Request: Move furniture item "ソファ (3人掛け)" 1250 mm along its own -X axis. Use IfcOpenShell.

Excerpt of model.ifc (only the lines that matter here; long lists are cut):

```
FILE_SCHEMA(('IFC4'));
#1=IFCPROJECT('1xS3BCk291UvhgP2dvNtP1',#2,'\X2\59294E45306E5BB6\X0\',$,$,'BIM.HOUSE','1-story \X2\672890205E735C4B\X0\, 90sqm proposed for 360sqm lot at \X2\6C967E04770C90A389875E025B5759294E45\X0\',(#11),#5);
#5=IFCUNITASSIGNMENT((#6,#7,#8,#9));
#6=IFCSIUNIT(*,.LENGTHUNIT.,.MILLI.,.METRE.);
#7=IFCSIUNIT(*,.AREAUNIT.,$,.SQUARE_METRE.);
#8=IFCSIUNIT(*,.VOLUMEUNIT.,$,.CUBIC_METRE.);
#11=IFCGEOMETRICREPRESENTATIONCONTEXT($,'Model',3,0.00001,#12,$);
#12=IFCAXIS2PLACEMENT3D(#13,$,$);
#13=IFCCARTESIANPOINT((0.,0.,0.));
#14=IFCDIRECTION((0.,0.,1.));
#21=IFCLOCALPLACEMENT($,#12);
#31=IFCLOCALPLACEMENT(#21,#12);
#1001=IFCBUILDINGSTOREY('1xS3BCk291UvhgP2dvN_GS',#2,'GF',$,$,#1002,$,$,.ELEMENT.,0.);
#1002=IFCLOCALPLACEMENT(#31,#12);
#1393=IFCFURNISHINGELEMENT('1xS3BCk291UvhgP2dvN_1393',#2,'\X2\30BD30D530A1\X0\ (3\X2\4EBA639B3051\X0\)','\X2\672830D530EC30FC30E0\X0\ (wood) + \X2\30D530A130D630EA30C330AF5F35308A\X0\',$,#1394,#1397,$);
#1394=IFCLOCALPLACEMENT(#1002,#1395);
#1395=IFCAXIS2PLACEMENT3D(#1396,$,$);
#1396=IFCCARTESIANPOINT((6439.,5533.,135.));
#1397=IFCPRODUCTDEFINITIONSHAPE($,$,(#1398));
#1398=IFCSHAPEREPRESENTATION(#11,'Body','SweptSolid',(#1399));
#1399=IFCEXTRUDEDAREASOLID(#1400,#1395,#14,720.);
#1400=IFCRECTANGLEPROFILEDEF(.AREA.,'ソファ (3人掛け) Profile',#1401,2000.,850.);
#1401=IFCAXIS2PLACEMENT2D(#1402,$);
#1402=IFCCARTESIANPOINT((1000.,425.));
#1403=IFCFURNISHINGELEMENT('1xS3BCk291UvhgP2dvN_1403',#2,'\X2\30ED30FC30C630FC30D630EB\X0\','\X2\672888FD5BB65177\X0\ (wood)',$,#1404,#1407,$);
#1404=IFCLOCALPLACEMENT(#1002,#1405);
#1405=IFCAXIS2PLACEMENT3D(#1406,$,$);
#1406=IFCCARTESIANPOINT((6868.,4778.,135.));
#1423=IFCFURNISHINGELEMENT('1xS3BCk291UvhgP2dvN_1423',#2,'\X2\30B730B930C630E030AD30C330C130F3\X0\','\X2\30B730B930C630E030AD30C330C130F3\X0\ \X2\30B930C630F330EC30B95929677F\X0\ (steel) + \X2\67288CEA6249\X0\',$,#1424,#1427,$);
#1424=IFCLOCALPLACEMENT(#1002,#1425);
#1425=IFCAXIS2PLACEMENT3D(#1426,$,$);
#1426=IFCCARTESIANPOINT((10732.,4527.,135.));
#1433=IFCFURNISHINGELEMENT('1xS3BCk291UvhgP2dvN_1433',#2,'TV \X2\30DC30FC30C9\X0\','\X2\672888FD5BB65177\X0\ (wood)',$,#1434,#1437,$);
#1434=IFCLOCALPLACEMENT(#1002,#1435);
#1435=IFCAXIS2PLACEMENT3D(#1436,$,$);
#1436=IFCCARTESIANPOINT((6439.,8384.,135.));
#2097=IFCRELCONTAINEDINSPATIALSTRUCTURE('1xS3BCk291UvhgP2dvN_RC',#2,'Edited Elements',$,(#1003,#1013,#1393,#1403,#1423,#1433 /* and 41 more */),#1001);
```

```python
import ifcopenshell
import ifcopenshell.api.geometry
import ifcopenshell.util.placement
import ifcopenshell.util.unit

model = ifcopenshell.open("model.ifc")
unit_scale = ifcopenshell.util.unit.calculate_unit_scale(model)

item = model.by_id(1393)
matrix = ifcopenshell.util.placement.get_local_placement(item.ObjectPlacement)
matrix[:3, 3] -= matrix[:3, 0] * 1.25 / unit_scale
ifcopenshell.api.geometry.edit_object_placement(model, product=item, matrix=matrix, is_si=False)

print(ifcopenshell.util.placement.get_local_placement(item.ObjectPlacement).round(3) + 0.0)

model.write("model-out.ifc")
```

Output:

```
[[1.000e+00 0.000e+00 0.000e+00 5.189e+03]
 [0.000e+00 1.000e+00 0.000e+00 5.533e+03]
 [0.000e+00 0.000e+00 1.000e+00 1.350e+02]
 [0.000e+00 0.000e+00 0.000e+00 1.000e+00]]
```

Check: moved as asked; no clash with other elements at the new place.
